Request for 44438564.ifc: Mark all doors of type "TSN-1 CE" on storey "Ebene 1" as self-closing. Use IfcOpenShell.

First a look at what the model holds.

```python
import ifcopenshell
import ifcopenshell.util.element

model = ifcopenshell.open("44438564.ifc")
print(model.schema)
storey = next(s for s in model.by_type("IfcBuildingStorey") if s.Name == "Ebene 1")
doors = [e for e in ifcopenshell.util.element.get_decomposition(storey) if e.is_a("IfcDoor")]
seen = {}
for e in doors:
    element_type = ifcopenshell.util.element.get_type(e)
    key = (element_type.Name if element_type != e and element_type else None, ifcopenshell.util.element.get_pset(e, "Pset_DoorCommon", "SelfClosing"))
    seen[key] = seen.get(key, 0) + 1
for (name, value), count in sorted(seen.items(), key=str):
    print(count, "x", name, "|", value)
```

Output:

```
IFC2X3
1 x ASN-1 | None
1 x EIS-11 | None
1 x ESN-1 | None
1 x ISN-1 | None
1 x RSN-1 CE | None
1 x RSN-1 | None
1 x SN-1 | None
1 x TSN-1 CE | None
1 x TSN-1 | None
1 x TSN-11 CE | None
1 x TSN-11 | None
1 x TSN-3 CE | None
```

```python
import ifcopenshell
import ifcopenshell.api.pset
import ifcopenshell.util.element

model = ifcopenshell.open("44438564.ifc")

storey = next(s for s in model.by_type("IfcBuildingStorey") if s.Name == "Ebene 1")
doors = [e for e in ifcopenshell.util.element.get_decomposition(storey) if e.is_a("IfcDoor")]

count = 0
for e in doors:
    element_type = ifcopenshell.util.element.get_type(e)
    if element_type in (None, e) or element_type.Name != "TSN-1 CE":
        continue
    # add_pset returns the element's existing set when there is one.
    pset = ifcopenshell.api.pset.add_pset(model, product=e, name="Pset_DoorCommon")
    ifcopenshell.api.pset.edit_pset(model, pset=pset, properties={"SelfClosing": True})
    count += 1

print(count, "doors updated")

model.write("44438564_v2.ifc")
```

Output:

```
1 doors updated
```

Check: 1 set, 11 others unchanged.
